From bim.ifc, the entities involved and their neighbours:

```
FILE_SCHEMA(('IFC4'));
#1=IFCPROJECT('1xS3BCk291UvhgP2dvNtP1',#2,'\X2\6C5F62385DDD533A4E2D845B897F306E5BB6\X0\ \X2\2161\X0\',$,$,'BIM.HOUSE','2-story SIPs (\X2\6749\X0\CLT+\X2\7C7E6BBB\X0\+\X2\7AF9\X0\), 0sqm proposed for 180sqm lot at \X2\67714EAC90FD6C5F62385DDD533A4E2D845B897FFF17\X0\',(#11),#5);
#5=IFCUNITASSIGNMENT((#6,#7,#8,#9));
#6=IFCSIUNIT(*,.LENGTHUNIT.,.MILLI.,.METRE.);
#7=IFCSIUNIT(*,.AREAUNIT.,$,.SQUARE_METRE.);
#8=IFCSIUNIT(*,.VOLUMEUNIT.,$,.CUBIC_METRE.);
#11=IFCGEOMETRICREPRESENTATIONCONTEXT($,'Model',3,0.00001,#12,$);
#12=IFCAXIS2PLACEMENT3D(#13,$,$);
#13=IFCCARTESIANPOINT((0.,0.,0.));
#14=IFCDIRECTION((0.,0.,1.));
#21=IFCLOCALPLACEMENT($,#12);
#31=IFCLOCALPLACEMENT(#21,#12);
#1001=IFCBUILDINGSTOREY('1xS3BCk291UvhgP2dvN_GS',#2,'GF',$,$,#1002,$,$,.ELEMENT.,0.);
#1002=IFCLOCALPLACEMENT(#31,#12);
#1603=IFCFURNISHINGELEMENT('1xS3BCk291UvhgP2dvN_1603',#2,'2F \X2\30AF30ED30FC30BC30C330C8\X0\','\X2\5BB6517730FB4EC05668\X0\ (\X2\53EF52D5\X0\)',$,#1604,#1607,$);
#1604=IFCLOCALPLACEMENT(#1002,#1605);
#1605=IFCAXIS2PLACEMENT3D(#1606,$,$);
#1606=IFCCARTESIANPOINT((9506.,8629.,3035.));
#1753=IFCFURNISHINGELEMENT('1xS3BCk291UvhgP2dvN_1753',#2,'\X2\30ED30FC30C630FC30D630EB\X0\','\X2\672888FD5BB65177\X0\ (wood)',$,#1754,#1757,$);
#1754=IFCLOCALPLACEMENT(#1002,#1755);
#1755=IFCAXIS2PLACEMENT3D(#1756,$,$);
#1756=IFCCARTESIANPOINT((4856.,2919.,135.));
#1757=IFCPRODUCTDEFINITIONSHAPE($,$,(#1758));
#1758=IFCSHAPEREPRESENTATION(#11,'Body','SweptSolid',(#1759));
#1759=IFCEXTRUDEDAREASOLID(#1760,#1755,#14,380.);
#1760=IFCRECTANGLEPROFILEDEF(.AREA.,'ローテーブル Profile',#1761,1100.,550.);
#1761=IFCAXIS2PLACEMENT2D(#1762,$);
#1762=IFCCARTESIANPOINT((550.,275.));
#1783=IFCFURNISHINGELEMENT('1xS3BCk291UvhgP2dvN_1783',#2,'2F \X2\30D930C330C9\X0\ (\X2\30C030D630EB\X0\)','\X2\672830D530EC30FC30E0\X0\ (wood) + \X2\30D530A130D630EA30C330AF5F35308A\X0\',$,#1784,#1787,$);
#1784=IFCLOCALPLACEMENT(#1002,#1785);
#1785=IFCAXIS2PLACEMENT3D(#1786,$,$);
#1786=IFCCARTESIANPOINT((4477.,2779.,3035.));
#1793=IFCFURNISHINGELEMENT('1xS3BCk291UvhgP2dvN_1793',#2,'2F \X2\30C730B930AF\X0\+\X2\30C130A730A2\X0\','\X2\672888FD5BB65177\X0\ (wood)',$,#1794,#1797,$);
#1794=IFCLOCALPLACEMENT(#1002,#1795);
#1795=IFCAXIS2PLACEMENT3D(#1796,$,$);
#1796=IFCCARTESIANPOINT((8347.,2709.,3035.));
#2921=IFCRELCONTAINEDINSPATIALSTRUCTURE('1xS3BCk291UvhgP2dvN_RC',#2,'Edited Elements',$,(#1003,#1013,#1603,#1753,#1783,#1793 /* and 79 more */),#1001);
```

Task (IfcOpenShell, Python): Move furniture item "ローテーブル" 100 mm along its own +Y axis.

```python
import ifcopenshell
import ifcopenshell.api.geometry
import ifcopenshell.util.placement

model = ifcopenshell.open("bim.ifc")

item = model.by_guid("1xS3BCk291UvhgP2dvN_1753")
matrix = ifcopenshell.util.placement.get_local_placement(item.ObjectPlacement)
matrix[:3, 3] += matrix[:3, 1] * 100.0
ifcopenshell.api.geometry.edit_object_placement(model, product=item, matrix=matrix, is_si=False)

print(ifcopenshell.util.placement.get_local_placement(item.ObjectPlacement).round(3) + 0.0)

model.write("bim_edited.ifc")
```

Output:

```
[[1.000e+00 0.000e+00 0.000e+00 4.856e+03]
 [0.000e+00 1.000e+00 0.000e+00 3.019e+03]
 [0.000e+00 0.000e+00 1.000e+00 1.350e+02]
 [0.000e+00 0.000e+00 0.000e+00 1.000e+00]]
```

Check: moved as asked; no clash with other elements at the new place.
